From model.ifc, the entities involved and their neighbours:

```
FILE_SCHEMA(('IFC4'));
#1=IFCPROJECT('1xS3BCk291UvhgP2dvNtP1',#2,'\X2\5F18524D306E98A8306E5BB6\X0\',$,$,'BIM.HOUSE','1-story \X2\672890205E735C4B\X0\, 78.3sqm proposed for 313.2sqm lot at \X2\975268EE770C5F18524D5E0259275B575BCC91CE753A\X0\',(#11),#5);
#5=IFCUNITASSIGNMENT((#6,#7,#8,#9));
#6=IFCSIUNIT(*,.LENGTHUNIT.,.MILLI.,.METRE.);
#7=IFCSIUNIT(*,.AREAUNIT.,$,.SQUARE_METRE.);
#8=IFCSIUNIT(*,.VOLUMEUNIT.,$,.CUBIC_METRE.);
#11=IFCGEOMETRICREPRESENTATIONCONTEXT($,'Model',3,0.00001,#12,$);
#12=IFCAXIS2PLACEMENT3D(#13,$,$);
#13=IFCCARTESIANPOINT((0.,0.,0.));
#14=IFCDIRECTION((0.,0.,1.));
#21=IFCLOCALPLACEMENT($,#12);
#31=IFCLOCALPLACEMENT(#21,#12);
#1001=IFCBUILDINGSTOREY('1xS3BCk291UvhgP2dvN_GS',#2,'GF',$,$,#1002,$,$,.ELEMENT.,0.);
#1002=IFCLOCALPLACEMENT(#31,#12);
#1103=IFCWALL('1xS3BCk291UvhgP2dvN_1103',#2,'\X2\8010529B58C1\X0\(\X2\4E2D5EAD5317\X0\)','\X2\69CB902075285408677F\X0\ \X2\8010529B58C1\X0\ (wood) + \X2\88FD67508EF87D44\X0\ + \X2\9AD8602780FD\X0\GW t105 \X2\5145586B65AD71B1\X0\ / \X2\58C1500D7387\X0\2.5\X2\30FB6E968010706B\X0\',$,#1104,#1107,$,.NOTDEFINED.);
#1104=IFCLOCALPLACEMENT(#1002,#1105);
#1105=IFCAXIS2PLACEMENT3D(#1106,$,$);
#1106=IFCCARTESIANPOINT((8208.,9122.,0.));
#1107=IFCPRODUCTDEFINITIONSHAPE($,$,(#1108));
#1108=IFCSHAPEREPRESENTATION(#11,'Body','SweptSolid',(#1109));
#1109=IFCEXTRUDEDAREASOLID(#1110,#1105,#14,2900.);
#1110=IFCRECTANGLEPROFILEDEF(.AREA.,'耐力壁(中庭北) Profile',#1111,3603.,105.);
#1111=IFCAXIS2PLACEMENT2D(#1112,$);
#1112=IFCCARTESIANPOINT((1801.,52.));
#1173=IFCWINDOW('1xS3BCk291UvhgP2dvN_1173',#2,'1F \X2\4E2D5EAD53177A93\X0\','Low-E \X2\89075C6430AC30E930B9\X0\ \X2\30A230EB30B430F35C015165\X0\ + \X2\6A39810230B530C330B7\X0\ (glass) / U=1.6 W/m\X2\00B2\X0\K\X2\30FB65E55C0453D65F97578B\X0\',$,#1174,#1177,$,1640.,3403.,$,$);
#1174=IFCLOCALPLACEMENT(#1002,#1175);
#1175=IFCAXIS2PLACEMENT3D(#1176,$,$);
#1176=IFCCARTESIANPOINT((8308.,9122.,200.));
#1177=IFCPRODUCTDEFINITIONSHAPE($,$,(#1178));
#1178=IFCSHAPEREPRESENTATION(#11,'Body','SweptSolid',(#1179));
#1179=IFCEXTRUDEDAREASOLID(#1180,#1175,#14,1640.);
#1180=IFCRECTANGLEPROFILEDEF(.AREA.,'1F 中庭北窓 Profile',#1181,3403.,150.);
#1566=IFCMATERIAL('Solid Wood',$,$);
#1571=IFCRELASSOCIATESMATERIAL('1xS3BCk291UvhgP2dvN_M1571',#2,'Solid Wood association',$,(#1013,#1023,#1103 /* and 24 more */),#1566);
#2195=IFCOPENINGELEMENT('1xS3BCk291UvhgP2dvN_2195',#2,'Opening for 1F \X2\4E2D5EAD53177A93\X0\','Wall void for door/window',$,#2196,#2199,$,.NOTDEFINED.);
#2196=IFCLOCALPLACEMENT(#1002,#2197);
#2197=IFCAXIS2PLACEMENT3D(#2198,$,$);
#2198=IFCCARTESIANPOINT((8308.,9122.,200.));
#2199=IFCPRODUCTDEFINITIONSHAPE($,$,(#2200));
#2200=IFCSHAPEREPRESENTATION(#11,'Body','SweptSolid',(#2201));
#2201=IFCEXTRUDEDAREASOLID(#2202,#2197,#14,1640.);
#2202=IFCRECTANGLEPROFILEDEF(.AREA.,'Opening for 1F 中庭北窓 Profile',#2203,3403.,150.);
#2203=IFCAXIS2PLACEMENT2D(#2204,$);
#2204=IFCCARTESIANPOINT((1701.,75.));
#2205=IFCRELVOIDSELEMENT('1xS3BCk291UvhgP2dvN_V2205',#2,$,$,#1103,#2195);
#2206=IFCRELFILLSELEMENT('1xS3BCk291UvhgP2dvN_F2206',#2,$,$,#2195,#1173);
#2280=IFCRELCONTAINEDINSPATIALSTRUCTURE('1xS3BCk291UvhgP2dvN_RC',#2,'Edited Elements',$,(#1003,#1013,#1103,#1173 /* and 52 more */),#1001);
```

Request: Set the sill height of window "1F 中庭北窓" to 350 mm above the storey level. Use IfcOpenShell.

```python
import numpy as np
import ifcopenshell
import ifcopenshell.api.geometry
import ifcopenshell.geom
import ifcopenshell.util.element
import ifcopenshell.util.placement
import ifcopenshell.util.shape
import ifcopenshell.util.unit

model = ifcopenshell.open("model.ifc")
unit_scale = ifcopenshell.util.unit.calculate_unit_scale(model)

window = model.by_id(1173)
opening = window.FillsVoids[0].RelatingOpeningElement
storey = ifcopenshell.util.element.get_container(window, ifc_class="IfcBuildingStorey")
level = ifcopenshell.util.placement.get_local_placement(storey.ObjectPlacement)[2, 3]

# The opening's origin need not be at the sill, so measure its lowest point.
shape = ifcopenshell.geom.create_shape(ifcopenshell.geom.settings(), opening)
bottom = ifcopenshell.util.shape.get_shape_bottom_elevation(shape, shape.geometry) / unit_scale
dz = level + 350.0 - bottom

shift = np.array([0.0, 0.0, dz])
# The window is not placed relative to its opening, so move both.
for product in (opening, window):
    matrix = ifcopenshell.util.placement.get_local_placement(product.ObjectPlacement)
    matrix[:3, 3] += shift
    ifcopenshell.api.geometry.edit_object_placement(model, product=product, matrix=matrix, is_si=False)

print(f"moved by {dz * unit_scale:+.3f} m")

model.write("model_edited.ifc")
```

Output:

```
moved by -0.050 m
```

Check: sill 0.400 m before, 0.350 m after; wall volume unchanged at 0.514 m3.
